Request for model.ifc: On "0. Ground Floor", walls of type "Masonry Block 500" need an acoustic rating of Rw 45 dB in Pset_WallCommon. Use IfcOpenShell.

First a look at what the model holds.

```python
import ifcopenshell
import ifcopenshell.util.element

model = ifcopenshell.open("model.ifc")
print(model.schema)
storey = next(s for s in model.by_type("IfcBuildingStorey") if s.Name == "0. Ground Floor")
walls = [e for e in ifcopenshell.util.element.get_decomposition(storey) if e.is_a("IfcWall")]
seen = {}
for e in walls:
    element_type = ifcopenshell.util.element.get_type(e)
    key = (element_type.Name if element_type != e and element_type else None, ifcopenshell.util.element.get_pset(e, "Pset_WallCommon", "AcousticRating"))
    seen[key] = seen.get(key, 0) + 1
for (name, value), count in sorted(seen.items(), key=str):
    print(count, "x", name, "|", value)
```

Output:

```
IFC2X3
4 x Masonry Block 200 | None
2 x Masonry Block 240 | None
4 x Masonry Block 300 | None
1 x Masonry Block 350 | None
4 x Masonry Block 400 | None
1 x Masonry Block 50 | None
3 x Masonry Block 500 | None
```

```python
import ifcopenshell
import ifcopenshell.api.pset
import ifcopenshell.util.element

model = ifcopenshell.open("model.ifc")

storey = next(s for s in model.by_type("IfcBuildingStorey") if s.Name == "0. Ground Floor")
walls = [e for e in ifcopenshell.util.element.get_decomposition(storey) if e.is_a("IfcWall")]

count = 0
for e in walls:
    element_type = ifcopenshell.util.element.get_type(e)
    if element_type in (None, e) or element_type.Name != "Masonry Block 500":
        continue
    # add_pset returns the element's existing set when there is one.
    pset = ifcopenshell.api.pset.add_pset(model, product=e, name="Pset_WallCommon")
    ifcopenshell.api.pset.edit_pset(model, pset=pset, properties={"AcousticRating": "Rw 45 dB"})
    count += 1

print(count, "walls updated")

model.write("model_updated.ifc")
```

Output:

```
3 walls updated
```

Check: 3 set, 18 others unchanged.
